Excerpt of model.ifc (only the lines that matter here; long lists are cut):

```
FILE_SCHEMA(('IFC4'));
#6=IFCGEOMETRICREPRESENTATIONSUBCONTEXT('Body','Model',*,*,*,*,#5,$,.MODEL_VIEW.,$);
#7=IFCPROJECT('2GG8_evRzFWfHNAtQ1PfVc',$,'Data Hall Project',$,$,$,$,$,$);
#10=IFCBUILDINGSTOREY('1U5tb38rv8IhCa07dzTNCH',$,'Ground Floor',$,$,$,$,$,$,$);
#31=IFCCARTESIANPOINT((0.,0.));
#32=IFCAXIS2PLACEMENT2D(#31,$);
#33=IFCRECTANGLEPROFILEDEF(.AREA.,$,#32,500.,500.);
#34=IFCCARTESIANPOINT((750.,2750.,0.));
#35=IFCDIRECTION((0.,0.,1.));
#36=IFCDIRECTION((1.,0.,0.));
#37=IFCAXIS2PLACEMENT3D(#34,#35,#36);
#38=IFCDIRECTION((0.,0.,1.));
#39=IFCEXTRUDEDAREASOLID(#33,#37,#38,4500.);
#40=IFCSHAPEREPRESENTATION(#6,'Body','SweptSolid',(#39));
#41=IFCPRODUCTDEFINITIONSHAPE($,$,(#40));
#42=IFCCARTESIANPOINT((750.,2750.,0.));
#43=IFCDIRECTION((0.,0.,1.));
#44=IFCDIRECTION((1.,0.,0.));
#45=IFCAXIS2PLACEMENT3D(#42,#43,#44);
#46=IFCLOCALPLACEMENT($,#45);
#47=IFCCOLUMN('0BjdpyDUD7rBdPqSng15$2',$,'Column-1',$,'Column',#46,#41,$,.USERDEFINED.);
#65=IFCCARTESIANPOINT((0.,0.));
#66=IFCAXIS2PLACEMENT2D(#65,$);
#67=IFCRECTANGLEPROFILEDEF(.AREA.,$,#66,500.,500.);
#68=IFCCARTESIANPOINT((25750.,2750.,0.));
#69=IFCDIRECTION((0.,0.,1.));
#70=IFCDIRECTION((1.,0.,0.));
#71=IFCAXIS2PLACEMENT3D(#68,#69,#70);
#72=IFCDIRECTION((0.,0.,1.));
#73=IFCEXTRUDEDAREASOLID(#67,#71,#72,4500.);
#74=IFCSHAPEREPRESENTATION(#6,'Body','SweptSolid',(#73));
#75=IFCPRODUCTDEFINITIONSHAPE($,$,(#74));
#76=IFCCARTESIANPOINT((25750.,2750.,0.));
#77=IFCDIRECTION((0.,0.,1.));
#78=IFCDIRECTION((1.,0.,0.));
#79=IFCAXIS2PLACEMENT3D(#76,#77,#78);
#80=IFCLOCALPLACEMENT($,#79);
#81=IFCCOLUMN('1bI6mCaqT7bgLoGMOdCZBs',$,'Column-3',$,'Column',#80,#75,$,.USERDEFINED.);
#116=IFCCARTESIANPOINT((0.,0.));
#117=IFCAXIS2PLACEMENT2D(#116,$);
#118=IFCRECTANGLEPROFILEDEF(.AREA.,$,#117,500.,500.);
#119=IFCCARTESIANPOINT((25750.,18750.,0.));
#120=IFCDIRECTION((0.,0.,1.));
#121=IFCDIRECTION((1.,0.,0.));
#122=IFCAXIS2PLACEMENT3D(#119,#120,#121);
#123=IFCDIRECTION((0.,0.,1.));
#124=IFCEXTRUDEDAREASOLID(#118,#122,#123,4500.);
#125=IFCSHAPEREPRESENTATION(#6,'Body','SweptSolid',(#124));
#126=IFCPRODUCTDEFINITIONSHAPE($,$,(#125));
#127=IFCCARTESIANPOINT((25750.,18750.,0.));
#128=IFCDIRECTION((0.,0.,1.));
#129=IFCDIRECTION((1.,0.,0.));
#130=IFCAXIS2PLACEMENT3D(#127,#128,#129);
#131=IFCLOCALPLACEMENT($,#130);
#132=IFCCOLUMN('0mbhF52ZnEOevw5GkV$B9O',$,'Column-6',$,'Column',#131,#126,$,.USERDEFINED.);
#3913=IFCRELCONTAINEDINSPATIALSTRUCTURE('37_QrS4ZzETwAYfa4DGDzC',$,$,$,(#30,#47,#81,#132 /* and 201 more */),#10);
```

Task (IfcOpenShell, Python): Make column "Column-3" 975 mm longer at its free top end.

```python
import ifcopenshell
import ifcopenshell.util.representation

model = ifcopenshell.open("model.ifc")

member = model.by_guid("1bI6mCaqT7bgLoGMOdCZBs")
change = 0.975

# The extrusion runs towards the end named, so only its depth changes.
body = ifcopenshell.util.representation.get_representation(member, "Model", "Body")
solid = body.Items[0]
old_length = solid.Depth
solid.Depth += change

print(f"length {old_length:g} -> {solid.Depth:g}")

model.write("model_v2.ifc")
```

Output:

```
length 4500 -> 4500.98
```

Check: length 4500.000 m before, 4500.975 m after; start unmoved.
